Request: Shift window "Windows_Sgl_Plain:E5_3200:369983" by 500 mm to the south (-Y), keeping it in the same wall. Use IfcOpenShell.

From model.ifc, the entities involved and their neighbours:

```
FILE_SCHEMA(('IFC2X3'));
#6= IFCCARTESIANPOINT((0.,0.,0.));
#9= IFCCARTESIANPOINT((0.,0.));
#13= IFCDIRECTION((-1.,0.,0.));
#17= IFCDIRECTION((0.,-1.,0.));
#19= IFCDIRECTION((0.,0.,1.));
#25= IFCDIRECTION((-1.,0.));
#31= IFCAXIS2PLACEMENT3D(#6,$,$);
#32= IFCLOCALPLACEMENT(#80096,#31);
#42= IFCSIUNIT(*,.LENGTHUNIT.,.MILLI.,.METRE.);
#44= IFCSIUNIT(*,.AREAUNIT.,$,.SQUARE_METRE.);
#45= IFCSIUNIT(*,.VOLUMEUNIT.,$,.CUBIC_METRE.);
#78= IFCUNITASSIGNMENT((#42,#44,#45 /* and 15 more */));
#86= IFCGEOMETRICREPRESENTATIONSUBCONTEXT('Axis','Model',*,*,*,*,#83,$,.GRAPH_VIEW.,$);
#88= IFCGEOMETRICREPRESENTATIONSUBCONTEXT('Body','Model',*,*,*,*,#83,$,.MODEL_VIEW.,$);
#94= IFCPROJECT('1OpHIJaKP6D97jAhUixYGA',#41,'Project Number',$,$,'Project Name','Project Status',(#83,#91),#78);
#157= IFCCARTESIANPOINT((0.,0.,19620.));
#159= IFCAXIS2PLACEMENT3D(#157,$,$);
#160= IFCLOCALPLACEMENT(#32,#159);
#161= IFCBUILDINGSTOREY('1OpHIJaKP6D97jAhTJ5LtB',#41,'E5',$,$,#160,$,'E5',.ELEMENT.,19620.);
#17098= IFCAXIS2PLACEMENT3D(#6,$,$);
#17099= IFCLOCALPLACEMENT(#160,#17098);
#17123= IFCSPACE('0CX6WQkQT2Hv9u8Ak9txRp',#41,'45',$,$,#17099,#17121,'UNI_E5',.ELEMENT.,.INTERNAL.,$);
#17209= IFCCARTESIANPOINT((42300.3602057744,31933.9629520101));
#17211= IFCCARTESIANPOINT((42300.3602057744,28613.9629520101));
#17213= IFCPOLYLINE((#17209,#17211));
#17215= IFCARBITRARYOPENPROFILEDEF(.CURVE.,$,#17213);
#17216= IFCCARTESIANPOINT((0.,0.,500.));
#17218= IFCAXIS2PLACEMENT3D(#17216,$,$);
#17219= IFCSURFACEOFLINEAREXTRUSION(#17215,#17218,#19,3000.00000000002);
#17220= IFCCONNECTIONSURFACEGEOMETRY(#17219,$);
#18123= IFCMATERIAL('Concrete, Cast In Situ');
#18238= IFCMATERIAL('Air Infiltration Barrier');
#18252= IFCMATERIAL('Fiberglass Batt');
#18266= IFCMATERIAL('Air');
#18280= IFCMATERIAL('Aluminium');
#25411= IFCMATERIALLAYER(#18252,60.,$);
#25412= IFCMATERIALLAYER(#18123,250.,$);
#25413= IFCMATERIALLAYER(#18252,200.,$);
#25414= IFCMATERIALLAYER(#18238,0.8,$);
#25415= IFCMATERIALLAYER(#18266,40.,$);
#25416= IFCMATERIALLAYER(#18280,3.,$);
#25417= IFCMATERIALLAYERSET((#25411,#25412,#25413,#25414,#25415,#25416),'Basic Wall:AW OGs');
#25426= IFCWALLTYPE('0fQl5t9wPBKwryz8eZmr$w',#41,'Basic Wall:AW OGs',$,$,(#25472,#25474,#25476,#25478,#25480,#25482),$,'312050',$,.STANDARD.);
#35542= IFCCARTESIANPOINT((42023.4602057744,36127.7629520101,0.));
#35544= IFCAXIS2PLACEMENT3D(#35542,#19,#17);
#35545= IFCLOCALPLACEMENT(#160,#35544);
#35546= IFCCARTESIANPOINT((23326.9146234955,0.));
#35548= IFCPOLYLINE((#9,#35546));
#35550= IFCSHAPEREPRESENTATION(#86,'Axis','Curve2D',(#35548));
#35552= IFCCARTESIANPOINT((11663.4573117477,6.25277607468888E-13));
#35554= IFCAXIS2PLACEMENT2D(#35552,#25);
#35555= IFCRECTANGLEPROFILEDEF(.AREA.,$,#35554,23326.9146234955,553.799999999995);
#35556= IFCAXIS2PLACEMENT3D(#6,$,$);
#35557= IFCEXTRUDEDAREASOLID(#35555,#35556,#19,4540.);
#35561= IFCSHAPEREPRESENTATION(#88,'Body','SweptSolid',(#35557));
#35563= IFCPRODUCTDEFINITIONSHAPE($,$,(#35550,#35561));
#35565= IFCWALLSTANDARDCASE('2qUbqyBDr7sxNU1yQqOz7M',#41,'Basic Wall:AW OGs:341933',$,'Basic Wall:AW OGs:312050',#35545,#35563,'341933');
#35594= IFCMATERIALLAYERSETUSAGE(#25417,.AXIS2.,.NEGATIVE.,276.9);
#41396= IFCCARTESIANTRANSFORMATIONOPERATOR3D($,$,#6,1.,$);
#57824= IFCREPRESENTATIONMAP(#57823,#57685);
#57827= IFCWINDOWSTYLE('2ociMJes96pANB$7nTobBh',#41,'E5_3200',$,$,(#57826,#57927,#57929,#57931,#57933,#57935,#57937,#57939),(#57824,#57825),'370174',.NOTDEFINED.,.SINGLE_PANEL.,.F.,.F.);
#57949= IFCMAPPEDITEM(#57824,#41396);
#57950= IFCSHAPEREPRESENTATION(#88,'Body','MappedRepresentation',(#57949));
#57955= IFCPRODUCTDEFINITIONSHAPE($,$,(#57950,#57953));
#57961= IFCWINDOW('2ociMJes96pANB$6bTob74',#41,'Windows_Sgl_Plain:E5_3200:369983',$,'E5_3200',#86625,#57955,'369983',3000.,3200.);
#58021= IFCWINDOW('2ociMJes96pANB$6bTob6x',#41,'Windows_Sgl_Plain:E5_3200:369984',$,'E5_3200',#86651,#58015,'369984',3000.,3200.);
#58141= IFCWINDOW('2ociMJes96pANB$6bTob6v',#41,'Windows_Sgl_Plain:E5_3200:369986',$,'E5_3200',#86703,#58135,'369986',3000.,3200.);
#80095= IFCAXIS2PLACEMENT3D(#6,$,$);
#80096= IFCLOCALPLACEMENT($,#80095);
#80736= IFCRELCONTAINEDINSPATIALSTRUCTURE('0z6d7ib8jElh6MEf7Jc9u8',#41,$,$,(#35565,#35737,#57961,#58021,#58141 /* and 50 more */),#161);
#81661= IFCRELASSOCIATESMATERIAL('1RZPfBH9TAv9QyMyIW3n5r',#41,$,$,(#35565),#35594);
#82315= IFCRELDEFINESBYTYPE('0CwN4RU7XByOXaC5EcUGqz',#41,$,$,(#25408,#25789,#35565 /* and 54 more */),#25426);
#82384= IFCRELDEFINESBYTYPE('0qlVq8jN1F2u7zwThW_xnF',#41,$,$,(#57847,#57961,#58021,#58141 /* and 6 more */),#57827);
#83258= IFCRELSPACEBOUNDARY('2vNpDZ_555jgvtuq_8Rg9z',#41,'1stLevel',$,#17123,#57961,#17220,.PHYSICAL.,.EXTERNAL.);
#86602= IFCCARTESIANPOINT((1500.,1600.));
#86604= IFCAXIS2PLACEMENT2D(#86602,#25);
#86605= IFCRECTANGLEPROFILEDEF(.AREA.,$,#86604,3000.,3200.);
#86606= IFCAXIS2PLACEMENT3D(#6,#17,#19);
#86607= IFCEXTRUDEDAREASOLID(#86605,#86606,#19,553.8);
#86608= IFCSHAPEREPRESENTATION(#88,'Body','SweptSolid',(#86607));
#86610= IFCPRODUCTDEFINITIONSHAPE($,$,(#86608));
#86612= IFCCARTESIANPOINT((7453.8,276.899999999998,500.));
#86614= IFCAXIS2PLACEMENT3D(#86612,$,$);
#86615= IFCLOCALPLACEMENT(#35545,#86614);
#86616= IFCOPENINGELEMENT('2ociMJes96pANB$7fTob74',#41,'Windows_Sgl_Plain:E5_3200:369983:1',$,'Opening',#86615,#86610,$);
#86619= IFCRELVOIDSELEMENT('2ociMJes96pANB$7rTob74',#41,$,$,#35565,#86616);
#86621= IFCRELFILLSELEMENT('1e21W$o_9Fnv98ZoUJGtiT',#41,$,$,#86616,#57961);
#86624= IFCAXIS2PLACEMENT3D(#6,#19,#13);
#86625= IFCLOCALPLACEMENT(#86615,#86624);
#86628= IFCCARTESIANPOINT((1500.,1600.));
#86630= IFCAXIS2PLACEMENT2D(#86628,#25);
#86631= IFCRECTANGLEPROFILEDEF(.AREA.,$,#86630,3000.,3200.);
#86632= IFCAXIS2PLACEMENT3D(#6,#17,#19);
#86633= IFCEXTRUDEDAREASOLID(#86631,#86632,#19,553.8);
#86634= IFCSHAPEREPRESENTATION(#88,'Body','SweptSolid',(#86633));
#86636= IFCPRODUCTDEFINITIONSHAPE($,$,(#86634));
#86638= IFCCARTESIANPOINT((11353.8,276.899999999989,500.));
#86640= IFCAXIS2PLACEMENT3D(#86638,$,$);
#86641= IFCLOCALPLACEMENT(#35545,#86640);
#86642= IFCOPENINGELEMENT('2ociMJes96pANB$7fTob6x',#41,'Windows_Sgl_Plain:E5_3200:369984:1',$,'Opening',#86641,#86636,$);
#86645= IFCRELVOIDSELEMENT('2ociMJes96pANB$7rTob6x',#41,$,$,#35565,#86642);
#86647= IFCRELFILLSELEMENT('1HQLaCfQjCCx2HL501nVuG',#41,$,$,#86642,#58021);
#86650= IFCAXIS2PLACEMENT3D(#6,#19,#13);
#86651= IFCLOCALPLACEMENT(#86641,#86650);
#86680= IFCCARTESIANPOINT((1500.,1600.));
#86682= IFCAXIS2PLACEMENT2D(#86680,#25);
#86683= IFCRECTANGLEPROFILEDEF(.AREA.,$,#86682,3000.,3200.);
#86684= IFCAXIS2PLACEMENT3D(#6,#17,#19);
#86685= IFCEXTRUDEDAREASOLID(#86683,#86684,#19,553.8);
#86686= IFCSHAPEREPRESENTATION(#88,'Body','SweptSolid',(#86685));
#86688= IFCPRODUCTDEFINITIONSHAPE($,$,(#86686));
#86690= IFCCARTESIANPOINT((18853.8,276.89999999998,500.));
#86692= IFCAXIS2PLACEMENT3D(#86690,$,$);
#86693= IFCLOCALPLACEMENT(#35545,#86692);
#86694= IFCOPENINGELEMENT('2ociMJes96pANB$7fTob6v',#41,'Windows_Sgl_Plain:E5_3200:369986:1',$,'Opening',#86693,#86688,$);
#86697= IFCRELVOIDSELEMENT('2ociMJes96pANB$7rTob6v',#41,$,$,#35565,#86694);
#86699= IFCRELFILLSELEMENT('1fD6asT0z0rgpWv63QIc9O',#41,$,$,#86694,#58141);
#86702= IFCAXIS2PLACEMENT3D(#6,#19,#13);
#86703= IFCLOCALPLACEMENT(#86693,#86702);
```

```python
import numpy as np
import ifcopenshell
import ifcopenshell.api.geometry
import ifcopenshell.util.placement
import ifcopenshell.util.unit

model = ifcopenshell.open("model.ifc")
unit_scale = ifcopenshell.util.unit.calculate_unit_scale(model)

window = model.by_id(57961)
opening = window.FillsVoids[0].RelatingOpeningElement
wall = opening.VoidsElements[0].RelatingBuildingElement

wall_matrix = ifcopenshell.util.placement.get_local_placement(wall.ObjectPlacement)
shift = wall_matrix[:3, 0] * 0.5 / unit_scale
before = ifcopenshell.util.placement.get_local_placement(window.ObjectPlacement)[:3, 3].copy()

# The window is placed relative to its opening, so it follows when the opening moves.
matrix = ifcopenshell.util.placement.get_local_placement(opening.ObjectPlacement)
matrix[:3, 3] += shift
ifcopenshell.api.geometry.edit_object_placement(
    model, product=opening, matrix=matrix, is_si=False, should_transform_children=True
)

# Space boundary surfaces are stored in each space's coordinates; move them too.
for rel in window.ProvidesBoundaries:
    if not rel.ConnectionGeometry:
        continue
    surface = rel.ConnectionGeometry.SurfaceOnRelatingElement
    space_matrix = ifcopenshell.util.placement.get_local_placement(rel.RelatingSpace.ObjectPlacement)
    point = np.array(surface.Position.Location.Coordinates) + space_matrix[:3, :3].T @ shift
    surface.Position = model.createIfcAxis2Placement3D(
        model.createIfcCartesianPoint(point.tolist()), surface.Position.Axis, surface.Position.RefDirection
    )

after = ifcopenshell.util.placement.get_local_placement(window.ObjectPlacement)[:3, 3]
print("window moved by", (after - before).round(3) + 0.0)

model.write("model_rev.ifc")
```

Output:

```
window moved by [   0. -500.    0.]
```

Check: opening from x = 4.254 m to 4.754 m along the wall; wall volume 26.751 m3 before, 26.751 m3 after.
